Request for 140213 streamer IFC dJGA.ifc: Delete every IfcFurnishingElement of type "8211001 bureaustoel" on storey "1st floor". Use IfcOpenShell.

First a look at what the model holds.

```python
import ifcopenshell
import ifcopenshell.util.element

model = ifcopenshell.open("140213 streamer IFC dJGA.ifc")
print(model.schema)
storey = next(s for s in model.by_type("IfcBuildingStorey") if s.Name == "1st floor")
furniture = [e for e in ifcopenshell.util.element.get_decomposition(storey) if e.is_a("IfcFurnishingElement")]
seen = {}
for e in furniture:
    element_type = ifcopenshell.util.element.get_type(e)
    name = element_type.Name if element_type not in (None, e) else None
    seen[name] = seen.get(name, 0) + 1
for name, count in sorted(seen.items(), key=str):
    print(count, "x", name)
```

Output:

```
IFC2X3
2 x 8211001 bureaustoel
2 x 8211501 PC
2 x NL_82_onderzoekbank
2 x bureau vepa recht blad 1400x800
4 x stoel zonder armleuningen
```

```python
import ifcopenshell
import ifcopenshell.api.root
import ifcopenshell.util.element

model = ifcopenshell.open("140213 streamer IFC dJGA.ifc")

storey = next(s for s in model.by_type("IfcBuildingStorey") if s.Name == "1st floor")
furniture = [e for e in ifcopenshell.util.element.get_decomposition(storey) if e.is_a("IfcFurnishingElement")]
targets = [e for e in furniture if (t := ifcopenshell.util.element.get_type(e)) not in (None, e) and t.Name == "8211001 bureaustoel"]

for e in targets:
    ifcopenshell.api.root.remove_product(model, product=e)
print(len(targets), "removed")

model.write("140213 streamer IFC dJGA-out.ifc")
```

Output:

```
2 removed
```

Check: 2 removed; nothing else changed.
